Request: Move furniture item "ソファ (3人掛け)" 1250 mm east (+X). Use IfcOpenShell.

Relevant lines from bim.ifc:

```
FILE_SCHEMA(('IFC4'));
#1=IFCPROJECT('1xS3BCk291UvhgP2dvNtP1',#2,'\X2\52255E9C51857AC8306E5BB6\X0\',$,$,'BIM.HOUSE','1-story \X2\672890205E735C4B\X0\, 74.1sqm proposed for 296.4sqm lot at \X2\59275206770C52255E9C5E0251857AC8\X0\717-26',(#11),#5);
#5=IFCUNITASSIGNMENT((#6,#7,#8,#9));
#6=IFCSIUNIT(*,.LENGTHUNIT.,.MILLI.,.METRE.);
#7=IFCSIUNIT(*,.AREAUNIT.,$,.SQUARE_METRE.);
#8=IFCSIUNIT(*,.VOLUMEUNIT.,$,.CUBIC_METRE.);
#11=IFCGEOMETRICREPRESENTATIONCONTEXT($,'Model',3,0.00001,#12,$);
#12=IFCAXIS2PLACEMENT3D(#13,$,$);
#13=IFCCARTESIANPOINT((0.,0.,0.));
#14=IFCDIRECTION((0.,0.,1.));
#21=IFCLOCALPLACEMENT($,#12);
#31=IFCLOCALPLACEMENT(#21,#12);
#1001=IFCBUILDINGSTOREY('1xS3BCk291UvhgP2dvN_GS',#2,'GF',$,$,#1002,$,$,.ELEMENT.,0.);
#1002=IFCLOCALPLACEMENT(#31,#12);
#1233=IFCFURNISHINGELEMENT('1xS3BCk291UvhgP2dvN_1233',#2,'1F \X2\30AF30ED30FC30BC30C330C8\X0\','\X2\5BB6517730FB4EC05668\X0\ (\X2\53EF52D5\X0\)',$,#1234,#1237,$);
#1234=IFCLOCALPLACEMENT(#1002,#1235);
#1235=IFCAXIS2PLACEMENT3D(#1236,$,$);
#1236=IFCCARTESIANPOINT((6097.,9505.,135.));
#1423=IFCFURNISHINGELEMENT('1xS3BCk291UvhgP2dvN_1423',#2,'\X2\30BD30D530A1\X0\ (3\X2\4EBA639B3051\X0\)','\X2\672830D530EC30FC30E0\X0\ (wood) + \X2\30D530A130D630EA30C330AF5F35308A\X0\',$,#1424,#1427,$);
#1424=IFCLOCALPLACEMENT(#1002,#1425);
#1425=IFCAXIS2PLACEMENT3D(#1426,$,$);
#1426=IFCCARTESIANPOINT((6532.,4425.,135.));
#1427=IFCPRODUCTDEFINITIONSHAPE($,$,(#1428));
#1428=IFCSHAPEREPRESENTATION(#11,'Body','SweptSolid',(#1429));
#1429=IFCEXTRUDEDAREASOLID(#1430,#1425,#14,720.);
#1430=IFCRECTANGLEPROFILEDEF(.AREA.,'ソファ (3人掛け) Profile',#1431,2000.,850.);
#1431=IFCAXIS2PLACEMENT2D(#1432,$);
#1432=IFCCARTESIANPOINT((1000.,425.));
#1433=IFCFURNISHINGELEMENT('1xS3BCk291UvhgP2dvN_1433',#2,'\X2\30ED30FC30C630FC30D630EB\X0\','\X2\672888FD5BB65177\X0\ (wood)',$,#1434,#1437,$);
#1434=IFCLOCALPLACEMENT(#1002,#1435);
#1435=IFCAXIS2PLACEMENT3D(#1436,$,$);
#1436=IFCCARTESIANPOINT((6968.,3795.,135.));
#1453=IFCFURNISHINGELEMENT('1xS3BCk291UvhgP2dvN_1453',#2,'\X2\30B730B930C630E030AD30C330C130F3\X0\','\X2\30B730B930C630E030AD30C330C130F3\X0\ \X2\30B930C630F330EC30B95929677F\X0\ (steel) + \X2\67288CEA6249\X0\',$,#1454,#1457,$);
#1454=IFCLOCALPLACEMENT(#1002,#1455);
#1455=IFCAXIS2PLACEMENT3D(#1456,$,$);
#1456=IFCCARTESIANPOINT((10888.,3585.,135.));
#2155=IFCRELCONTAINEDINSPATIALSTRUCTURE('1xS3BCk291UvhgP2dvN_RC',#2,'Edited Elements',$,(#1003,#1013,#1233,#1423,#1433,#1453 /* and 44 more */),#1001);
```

```python
import ifcopenshell
import ifcopenshell.api.geometry
import ifcopenshell.util.placement

model = ifcopenshell.open("bim.ifc")

item = model.by_guid("1xS3BCk291UvhgP2dvN_1423")
matrix = ifcopenshell.util.placement.get_local_placement(item.ObjectPlacement)
matrix[0, 3] += 1250.0
ifcopenshell.api.geometry.edit_object_placement(model, product=item, matrix=matrix, is_si=False)

print(ifcopenshell.util.placement.get_local_placement(item.ObjectPlacement).round(3) + 0.0)

model.write("bim_updated.ifc")
```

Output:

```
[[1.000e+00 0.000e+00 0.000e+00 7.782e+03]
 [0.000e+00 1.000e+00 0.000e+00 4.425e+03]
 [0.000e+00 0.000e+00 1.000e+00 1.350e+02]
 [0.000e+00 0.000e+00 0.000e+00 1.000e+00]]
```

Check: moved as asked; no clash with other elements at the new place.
